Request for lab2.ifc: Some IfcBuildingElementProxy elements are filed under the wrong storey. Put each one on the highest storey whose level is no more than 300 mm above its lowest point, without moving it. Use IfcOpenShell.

First a look at what the model holds.

```python
import ifcopenshell
import ifcopenshell.util.element
import ifcopenshell.util.placement

model = ifcopenshell.open("lab2.ifc")
print(model.schema)
for storey in model.by_type("IfcBuildingStorey"):
    level = ifcopenshell.util.placement.get_storey_elevation(storey)
    count = sum(e.is_a("IfcBuildingElementProxy") for e in ifcopenshell.util.element.get_contained(storey))
    print(storey.id(), storey.Name, round(level, 3), count, sep=" | ")
```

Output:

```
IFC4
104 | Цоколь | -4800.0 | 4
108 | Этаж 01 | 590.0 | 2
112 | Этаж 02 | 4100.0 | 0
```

```python
import ifcopenshell
import ifcopenshell.api.spatial
import ifcopenshell.geom
import ifcopenshell.util.element
import ifcopenshell.util.placement
import ifcopenshell.util.shape
import ifcopenshell.util.unit

model = ifcopenshell.open("lab2.ifc")
unit_scale = ifcopenshell.util.unit.calculate_unit_scale(model)
settings = ifcopenshell.geom.settings()

levels = sorted(
    ((ifcopenshell.util.placement.get_storey_elevation(s) * unit_scale, s) for s in model.by_type("IfcBuildingStorey")),
    key=lambda pair: pair[0],
)

for e in model.by_type("IfcBuildingElementProxy"):
    current = e.ContainedInStructure[0].RelatingStructure if e.ContainedInStructure else None
    if current is None or not current.is_a("IfcBuildingStorey"):
        continue
    shape = ifcopenshell.geom.create_shape(settings, e)
    bottom = ifcopenshell.util.shape.get_shape_bottom_elevation(shape, shape.geometry)
    below = [s for level, s in levels if level <= bottom + 0.3]
    storey = below[-1] if below else levels[0][1]
    if storey != current:
        # assign_container keeps the world position.
        ifcopenshell.api.spatial.assign_container(model, products=[e], relating_structure=storey)
        print(e.id(), current.Name, "->", storey.Name)

model.write("lab2_v2.ifc")
```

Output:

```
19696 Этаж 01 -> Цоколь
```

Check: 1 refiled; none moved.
